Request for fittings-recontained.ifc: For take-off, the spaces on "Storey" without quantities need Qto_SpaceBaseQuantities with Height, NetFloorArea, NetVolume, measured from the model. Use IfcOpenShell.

First a look at what the model holds.

```python
import ifcopenshell
import ifcopenshell.util.element
import ifcopenshell.util.unit

model = ifcopenshell.open("fittings-recontained.ifc")
print(model.schema)
for unit_type in ("LENGTHUNIT", "AREAUNIT", "VOLUMEUNIT"):
    print(unit_type, ifcopenshell.util.unit.calculate_unit_scale(model, unit_type))
storey = next(s for s in model.by_type("IfcBuildingStorey") if s.Name == "Storey")
spaces = [e for e in ifcopenshell.util.element.get_decomposition(storey) if e.is_a("IfcSpace")]
for e in sorted(spaces, key=lambda e: e.id()):
    print(e.id(), e.is_a(), e.Name, list(ifcopenshell.util.element.get_psets(e, qtos_only=True)), sep=" | ")
```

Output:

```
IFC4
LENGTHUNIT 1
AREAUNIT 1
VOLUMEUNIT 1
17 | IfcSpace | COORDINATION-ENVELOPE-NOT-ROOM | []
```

```python
import ifcopenshell
import ifcopenshell.api.pset
import ifcopenshell.geom
import ifcopenshell.util.element
import ifcopenshell.util.shape
import ifcopenshell.util.unit

model = ifcopenshell.open("fittings-recontained.ifc")
unit_scale = ifcopenshell.util.unit.calculate_unit_scale(model)
area_scale = ifcopenshell.util.unit.calculate_unit_scale(model, "AREAUNIT")
volume_scale = ifcopenshell.util.unit.calculate_unit_scale(model, "VOLUMEUNIT")
settings = ifcopenshell.geom.settings()

storey = next(s for s in model.by_type("IfcBuildingStorey") if s.Name == "Storey")
spaces = [e for e in ifcopenshell.util.element.get_decomposition(storey) if e.is_a("IfcSpace")]

for e in sorted(spaces, key=lambda e: e.id()):
    if ifcopenshell.util.element.get_psets(e, qtos_only=True, should_inherit=False):
        continue
    # Geometry comes back in metres, in the element's own axes.
    shape = ifcopenshell.geom.create_shape(settings, e)
    values = {
        "Height": ifcopenshell.util.shape.get_z(shape.geometry) / unit_scale,
        "NetFloorArea": ifcopenshell.util.shape.get_footprint_area(shape.geometry) / area_scale,
        "NetVolume": ifcopenshell.util.shape.get_volume(shape.geometry) / volume_scale,
    }
    qto = ifcopenshell.api.pset.add_qto(model, product=e, name="Qto_SpaceBaseQuantities")
    ifcopenshell.api.pset.edit_qto(model, qto=qto, properties=values)
    print(e.id(), {k: round(v, 3) for k, v in values.items()})

model.write("fittings-recontained_updated.ifc")
```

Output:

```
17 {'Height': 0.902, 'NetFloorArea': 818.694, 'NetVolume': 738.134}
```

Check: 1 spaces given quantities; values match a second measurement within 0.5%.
